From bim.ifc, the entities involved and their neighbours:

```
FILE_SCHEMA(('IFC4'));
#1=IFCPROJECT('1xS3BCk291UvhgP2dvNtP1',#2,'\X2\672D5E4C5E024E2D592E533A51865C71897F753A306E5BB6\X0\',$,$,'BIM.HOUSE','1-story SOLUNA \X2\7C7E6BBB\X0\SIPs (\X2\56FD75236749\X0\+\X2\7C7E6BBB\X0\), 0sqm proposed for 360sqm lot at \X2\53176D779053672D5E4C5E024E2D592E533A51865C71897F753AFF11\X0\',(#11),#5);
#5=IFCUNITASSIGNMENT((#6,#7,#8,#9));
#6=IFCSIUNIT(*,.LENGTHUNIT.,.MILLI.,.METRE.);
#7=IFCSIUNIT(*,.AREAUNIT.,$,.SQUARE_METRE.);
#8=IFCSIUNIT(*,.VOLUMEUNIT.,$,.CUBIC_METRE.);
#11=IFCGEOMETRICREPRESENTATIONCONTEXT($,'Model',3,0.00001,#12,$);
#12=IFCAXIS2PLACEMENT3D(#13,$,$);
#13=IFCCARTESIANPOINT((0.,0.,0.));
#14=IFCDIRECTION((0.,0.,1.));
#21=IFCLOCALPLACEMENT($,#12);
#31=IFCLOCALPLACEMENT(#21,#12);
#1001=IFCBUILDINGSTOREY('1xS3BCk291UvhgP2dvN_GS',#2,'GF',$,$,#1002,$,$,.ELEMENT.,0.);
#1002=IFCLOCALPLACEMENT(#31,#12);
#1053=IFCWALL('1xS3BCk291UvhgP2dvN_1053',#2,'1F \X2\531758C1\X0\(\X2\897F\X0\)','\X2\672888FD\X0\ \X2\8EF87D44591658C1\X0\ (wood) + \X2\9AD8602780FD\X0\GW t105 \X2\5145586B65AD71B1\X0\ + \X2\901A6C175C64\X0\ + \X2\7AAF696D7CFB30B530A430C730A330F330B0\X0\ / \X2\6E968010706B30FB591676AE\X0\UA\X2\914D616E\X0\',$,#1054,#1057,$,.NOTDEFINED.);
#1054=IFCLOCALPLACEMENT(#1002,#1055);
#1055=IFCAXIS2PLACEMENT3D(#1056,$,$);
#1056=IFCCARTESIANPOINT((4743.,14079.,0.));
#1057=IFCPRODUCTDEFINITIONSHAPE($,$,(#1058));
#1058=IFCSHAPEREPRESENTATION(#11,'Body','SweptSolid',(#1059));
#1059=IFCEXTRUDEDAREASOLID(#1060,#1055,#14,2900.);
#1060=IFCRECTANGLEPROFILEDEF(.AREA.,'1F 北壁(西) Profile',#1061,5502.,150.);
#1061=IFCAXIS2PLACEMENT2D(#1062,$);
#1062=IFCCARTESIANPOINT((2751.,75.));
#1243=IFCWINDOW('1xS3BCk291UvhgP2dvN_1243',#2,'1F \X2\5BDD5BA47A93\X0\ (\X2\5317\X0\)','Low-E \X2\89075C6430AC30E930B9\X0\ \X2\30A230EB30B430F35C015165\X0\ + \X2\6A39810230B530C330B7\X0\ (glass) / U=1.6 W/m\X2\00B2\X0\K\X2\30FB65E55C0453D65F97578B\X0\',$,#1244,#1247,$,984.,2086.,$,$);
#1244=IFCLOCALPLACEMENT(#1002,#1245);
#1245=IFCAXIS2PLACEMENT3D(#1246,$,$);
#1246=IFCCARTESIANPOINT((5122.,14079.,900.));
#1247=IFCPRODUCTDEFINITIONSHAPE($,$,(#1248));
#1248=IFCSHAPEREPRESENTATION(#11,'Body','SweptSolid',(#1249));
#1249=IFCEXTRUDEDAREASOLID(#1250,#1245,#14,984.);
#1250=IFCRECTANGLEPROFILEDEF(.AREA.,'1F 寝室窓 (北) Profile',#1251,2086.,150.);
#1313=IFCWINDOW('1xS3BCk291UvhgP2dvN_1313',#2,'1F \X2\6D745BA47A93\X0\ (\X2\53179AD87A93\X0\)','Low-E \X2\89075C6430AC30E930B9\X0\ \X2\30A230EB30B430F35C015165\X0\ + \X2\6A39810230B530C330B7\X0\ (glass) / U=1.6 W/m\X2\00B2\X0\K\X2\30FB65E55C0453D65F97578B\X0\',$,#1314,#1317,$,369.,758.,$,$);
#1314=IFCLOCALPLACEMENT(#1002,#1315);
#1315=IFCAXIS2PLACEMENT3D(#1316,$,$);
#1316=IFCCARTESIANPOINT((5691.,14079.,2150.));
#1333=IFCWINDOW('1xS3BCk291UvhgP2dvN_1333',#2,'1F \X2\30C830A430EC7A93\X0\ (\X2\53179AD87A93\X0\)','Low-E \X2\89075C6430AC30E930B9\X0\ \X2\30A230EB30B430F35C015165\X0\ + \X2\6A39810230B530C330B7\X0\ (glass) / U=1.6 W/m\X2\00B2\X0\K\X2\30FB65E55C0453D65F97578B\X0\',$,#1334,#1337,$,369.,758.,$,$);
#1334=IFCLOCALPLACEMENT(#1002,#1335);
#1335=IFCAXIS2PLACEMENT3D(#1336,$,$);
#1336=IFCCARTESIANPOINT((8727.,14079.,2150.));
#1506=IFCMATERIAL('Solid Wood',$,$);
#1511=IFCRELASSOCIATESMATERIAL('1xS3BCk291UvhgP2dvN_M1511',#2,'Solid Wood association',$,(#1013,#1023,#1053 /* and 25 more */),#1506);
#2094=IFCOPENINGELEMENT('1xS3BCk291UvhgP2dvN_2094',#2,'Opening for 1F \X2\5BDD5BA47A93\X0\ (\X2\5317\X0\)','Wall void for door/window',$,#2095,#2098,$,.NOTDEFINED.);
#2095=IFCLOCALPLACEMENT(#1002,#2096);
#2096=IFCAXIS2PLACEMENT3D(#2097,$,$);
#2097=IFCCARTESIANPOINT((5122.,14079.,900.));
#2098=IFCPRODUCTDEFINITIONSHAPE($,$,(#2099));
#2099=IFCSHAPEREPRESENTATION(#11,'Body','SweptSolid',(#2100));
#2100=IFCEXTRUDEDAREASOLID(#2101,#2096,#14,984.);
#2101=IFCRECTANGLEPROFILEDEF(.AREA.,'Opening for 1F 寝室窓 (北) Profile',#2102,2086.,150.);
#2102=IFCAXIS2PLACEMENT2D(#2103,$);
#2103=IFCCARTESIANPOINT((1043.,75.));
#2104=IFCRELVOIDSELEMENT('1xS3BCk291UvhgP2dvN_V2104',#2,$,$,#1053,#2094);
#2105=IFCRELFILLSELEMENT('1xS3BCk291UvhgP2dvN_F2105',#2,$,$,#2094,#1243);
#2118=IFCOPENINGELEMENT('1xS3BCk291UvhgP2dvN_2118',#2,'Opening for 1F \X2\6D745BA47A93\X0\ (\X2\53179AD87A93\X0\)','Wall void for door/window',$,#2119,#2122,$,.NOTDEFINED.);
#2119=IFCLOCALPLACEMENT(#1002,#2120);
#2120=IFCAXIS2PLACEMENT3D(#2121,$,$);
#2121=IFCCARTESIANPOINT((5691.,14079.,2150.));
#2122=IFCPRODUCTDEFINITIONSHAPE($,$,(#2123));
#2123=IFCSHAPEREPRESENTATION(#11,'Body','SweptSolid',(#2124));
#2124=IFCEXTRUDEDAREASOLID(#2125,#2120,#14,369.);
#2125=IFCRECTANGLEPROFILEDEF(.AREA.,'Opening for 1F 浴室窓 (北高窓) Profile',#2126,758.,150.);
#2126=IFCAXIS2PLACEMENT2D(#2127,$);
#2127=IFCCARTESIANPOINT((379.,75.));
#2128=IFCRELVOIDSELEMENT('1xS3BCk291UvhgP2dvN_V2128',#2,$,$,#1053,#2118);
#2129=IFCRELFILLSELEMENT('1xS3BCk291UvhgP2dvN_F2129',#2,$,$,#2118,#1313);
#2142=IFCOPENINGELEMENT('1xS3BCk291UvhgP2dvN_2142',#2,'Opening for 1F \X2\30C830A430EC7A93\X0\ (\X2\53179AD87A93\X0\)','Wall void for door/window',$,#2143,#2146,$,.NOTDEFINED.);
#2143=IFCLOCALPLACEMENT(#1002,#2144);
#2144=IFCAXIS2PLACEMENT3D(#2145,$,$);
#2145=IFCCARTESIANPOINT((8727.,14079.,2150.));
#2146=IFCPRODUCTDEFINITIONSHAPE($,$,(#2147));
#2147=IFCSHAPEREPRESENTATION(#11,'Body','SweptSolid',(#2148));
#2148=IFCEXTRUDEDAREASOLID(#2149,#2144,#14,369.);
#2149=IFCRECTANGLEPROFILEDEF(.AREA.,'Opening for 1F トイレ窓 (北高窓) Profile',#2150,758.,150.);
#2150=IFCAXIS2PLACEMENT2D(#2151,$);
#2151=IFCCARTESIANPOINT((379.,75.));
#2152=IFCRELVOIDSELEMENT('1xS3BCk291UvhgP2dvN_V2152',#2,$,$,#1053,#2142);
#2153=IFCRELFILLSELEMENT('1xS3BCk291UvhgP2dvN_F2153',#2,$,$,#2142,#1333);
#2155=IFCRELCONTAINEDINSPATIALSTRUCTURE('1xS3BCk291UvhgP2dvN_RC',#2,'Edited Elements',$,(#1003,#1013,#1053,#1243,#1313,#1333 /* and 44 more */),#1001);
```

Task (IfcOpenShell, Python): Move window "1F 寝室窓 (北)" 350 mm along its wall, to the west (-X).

```python
import ifcopenshell
import ifcopenshell.api.geometry
import ifcopenshell.util.placement
import ifcopenshell.util.unit

model = ifcopenshell.open("bim.ifc")
unit_scale = ifcopenshell.util.unit.calculate_unit_scale(model)

window = model.by_guid("1xS3BCk291UvhgP2dvN_1243")
opening = window.FillsVoids[0].RelatingOpeningElement
wall = opening.VoidsElements[0].RelatingBuildingElement

wall_matrix = ifcopenshell.util.placement.get_local_placement(wall.ObjectPlacement)
shift = wall_matrix[:3, 0] * -0.35 / unit_scale
before = ifcopenshell.util.placement.get_local_placement(window.ObjectPlacement)[:3, 3].copy()

# The window is not placed relative to its opening, so move both.
for product in (opening, window):
    matrix = ifcopenshell.util.placement.get_local_placement(product.ObjectPlacement)
    matrix[:3, 3] += shift
    ifcopenshell.api.geometry.edit_object_placement(model, product=product, matrix=matrix, is_si=False)

after = ifcopenshell.util.placement.get_local_placement(window.ObjectPlacement)[:3, 3]
print("window moved by", (after - before).round(3) + 0.0)

model.write("bim_rev.ifc")
```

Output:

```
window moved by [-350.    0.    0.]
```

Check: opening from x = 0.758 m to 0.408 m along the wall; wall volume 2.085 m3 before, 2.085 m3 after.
